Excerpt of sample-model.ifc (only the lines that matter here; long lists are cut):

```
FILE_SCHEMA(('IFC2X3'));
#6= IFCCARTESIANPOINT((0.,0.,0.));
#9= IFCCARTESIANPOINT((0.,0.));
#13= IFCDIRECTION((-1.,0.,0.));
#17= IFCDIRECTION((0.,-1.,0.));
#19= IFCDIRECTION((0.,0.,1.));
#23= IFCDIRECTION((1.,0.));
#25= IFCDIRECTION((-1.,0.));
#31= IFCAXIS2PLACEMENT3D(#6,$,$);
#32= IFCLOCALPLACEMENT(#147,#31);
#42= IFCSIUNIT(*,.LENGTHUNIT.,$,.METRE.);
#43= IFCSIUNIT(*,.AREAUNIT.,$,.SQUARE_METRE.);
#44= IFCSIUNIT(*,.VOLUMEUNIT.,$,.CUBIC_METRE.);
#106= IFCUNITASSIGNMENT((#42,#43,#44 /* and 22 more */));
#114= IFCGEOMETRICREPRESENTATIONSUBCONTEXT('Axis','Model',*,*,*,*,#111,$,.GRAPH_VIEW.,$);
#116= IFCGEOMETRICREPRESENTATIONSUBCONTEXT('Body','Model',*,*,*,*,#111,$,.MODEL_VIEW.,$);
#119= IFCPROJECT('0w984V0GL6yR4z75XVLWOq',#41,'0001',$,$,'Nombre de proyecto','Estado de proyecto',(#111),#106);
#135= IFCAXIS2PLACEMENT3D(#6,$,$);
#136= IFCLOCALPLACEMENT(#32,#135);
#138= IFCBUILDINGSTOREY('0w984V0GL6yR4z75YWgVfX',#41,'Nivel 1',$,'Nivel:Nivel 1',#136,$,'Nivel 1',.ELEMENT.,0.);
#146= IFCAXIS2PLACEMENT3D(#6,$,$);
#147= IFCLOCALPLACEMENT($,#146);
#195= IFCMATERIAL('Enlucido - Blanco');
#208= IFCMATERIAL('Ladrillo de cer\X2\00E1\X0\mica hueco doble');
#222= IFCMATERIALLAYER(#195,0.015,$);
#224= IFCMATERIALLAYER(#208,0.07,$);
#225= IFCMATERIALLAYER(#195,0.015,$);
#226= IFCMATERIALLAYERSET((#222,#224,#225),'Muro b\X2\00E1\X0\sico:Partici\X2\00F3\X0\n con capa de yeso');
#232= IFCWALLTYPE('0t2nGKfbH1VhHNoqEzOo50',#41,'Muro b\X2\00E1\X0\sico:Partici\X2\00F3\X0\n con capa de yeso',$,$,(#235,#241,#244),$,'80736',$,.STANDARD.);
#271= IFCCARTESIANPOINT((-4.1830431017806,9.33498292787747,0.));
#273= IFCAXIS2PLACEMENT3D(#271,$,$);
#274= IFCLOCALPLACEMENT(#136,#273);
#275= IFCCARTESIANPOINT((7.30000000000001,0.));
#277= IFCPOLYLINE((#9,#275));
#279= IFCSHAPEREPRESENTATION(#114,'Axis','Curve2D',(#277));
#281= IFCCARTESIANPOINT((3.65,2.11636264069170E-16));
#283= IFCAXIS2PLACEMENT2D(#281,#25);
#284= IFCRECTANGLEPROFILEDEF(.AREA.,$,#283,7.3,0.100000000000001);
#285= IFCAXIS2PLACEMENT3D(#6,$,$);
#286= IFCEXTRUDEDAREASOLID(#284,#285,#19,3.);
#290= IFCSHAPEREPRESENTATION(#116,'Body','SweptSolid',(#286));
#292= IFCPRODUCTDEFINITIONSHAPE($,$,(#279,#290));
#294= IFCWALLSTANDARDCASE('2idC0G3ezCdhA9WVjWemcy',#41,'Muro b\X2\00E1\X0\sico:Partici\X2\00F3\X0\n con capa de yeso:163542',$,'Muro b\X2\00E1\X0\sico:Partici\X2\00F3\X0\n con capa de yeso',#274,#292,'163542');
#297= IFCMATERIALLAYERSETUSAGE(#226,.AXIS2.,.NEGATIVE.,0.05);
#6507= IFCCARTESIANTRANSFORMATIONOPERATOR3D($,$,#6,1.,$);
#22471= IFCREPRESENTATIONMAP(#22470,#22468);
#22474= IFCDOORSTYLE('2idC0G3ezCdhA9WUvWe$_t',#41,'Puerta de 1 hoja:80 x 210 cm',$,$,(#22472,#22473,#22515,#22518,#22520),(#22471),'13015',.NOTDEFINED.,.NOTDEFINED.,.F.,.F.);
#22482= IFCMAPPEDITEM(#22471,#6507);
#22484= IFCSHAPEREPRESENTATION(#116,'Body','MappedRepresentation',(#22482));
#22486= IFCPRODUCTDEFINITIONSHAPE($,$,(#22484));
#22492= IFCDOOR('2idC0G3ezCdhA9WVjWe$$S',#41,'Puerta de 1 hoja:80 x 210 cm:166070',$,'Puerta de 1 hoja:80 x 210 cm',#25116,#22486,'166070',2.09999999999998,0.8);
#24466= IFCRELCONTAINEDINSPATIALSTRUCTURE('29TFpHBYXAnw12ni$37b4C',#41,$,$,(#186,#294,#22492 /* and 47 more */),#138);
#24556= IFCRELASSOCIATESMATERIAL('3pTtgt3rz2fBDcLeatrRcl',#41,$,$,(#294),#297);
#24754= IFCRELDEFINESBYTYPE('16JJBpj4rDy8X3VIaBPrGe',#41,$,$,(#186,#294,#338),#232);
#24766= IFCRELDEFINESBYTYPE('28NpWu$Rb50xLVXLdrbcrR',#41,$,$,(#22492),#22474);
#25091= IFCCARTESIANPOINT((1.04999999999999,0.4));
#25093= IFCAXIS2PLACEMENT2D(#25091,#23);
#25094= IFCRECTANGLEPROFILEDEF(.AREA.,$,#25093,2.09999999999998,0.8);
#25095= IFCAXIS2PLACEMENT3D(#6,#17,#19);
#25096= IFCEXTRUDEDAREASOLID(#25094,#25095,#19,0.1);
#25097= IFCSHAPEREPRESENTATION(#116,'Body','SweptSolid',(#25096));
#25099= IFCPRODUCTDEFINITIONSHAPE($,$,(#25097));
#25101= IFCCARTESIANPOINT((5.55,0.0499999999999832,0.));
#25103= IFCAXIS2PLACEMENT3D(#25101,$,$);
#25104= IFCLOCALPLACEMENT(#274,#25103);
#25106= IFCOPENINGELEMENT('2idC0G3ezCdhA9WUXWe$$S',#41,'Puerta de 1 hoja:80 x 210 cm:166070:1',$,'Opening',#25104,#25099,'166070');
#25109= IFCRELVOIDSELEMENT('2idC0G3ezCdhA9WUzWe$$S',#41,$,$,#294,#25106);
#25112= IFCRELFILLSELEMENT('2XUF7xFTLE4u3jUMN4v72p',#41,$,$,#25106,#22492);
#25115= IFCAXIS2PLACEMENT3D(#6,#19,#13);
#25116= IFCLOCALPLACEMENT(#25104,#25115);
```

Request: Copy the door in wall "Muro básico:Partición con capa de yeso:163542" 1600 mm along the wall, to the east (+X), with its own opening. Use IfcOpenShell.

```python
import ifcopenshell
import ifcopenshell.api.feature
import ifcopenshell.api.geometry
import ifcopenshell.api.root
import ifcopenshell.geom
import ifcopenshell.util.element
import ifcopenshell.util.placement
import ifcopenshell.util.shape
import ifcopenshell.util.unit

model = ifcopenshell.open("sample-model.ifc")
unit_scale = ifcopenshell.util.unit.calculate_unit_scale(model)
settings = ifcopenshell.geom.settings()


def volume(element):
    """Net volume in cubic metres, openings subtracted."""
    shape = ifcopenshell.geom.create_shape(settings, element)
    return ifcopenshell.util.shape.get_volume(shape.geometry)


def reuse_history(source, copy):
    """copy_class also copies each property set's owner history, people and application; keep the originals."""
    for rel in copy.IsDefinedBy:
        if rel.is_a("IfcRelDefinesByProperties") and (history := rel.RelatingPropertyDefinition.OwnerHistory):
            rel.RelatingPropertyDefinition.OwnerHistory = source.OwnerHistory
            ifcopenshell.util.element.remove_deep2(model, history)


door = model.by_id(22492)
opening = door.FillsVoids[0].RelatingOpeningElement
wall = opening.VoidsElements[0].RelatingBuildingElement
before = volume(wall)
shift = ifcopenshell.util.placement.get_local_placement(wall.ObjectPlacement)[:3, 0] * 1.6 / unit_scale

# copy_class copies the void relationship, type, container and properties, but no geometry.
new_opening = ifcopenshell.api.root.copy_class(model, product=opening)
new_opening.Representation = ifcopenshell.util.element.copy_deep(
    model, opening.Representation, exclude=["IfcGeometricRepresentationContext", "IfcRepresentationMap"]
)
new_opening.Name = "Puerta de 1 hoja:80 x 210 cm"
new_opening.Tag = None
new_door = ifcopenshell.api.root.copy_class(model, product=door)
new_door.Representation = ifcopenshell.util.element.copy_deep(
    model, door.Representation, exclude=["IfcGeometricRepresentationContext", "IfcRepresentationMap"]
)
new_door.Name = "Puerta de 1 hoja:80 x 210 cm"
new_door.Tag = None
reuse_history(door, new_door)
fills = ifcopenshell.api.feature.add_filling(model, opening=new_opening, element=new_door)
fills.OwnerHistory = new_door.OwnerHistory  # required in IFC2X3

for old, new in ((opening, new_opening), (door, new_door)):
    matrix = ifcopenshell.util.placement.get_local_placement(old.ObjectPlacement)
    matrix[:3, 3] += shift
    ifcopenshell.api.geometry.edit_object_placement(model, product=new, matrix=matrix, is_si=False)

after = volume(wall)

print(f"wall volume {before:.3f} -> {after:.3f} m3")

model.write("sample-model_edited.ifc")
```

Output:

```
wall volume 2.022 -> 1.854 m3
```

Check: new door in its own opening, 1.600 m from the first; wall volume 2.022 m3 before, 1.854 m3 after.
